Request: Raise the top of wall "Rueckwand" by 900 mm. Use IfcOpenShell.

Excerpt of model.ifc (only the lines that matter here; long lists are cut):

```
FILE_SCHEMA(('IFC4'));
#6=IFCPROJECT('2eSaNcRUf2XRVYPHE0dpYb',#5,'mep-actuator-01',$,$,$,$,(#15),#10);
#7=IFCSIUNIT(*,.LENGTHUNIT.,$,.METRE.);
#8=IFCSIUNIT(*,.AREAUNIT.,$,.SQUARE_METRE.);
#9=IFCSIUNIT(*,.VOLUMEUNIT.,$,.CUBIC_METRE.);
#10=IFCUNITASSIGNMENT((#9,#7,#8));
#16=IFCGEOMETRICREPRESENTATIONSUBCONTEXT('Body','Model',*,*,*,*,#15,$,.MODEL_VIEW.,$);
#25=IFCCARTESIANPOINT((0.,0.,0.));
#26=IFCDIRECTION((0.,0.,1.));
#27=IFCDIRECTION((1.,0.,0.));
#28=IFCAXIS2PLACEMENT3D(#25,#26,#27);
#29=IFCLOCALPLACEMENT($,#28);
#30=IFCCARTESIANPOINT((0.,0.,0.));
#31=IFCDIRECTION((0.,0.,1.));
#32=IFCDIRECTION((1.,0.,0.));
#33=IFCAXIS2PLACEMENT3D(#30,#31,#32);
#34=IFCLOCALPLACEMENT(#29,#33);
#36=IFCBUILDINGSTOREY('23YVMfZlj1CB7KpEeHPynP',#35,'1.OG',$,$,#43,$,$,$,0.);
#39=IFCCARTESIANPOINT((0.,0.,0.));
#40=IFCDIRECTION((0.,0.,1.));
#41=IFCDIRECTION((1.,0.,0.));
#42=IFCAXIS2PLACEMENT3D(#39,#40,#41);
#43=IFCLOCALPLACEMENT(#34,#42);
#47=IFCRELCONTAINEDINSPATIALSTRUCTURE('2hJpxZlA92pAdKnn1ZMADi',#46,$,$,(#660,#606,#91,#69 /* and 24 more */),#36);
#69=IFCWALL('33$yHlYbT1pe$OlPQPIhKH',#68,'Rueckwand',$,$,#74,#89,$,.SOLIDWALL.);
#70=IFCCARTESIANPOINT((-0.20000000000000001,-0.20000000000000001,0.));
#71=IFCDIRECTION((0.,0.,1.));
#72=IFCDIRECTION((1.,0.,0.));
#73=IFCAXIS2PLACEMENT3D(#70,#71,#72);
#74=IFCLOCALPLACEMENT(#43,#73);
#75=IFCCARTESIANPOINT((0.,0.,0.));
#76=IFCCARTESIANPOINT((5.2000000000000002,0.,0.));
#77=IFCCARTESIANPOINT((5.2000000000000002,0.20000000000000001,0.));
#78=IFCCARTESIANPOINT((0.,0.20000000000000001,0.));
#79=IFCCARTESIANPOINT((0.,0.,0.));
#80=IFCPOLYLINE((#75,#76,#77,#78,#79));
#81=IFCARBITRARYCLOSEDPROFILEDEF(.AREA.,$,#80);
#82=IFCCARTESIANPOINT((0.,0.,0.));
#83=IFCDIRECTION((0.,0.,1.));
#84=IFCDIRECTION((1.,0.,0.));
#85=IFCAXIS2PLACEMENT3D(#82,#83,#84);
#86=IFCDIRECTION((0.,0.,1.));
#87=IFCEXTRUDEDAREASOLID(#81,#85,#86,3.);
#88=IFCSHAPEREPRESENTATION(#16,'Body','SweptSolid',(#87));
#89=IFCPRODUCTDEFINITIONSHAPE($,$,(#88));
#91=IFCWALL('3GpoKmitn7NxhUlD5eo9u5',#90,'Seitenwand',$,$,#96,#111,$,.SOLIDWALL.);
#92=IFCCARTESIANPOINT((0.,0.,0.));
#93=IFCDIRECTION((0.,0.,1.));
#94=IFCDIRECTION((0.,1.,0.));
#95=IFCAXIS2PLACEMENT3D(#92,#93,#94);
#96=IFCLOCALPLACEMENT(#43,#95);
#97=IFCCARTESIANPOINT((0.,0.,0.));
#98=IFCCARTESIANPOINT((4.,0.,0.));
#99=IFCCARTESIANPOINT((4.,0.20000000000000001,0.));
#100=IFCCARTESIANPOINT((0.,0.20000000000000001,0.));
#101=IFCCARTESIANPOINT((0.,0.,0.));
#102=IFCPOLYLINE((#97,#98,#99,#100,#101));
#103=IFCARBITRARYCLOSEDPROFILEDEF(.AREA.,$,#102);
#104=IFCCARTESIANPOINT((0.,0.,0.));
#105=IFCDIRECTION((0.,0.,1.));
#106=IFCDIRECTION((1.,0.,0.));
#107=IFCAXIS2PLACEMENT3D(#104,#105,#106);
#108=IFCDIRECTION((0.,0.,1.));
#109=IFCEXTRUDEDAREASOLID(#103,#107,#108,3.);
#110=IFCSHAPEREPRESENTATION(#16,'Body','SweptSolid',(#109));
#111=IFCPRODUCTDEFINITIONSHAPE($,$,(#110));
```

```python
import ifcopenshell
import ifcopenshell.geom
import ifcopenshell.util.representation
import ifcopenshell.util.shape

model = ifcopenshell.open("model.ifc")
settings = ifcopenshell.geom.settings()


def volume(element):
    """Net volume in cubic metres, openings subtracted."""
    shape = ifcopenshell.geom.create_shape(settings, element)
    return ifcopenshell.util.shape.get_volume(shape.geometry)


wall = model.by_guid("33$yHlYbT1pe$OlPQPIhKH")
before = volume(wall)

body = ifcopenshell.util.representation.get_representation(wall, "Model", "Body")
solid = body.Items[0]
old_height = solid.Depth
solid.Depth += 0.9
after = volume(wall)

print(f"height {old_height:g} -> {solid.Depth:g}, volume {before:.3f} -> {after:.3f} m3")

model.write("model-out.ifc")
```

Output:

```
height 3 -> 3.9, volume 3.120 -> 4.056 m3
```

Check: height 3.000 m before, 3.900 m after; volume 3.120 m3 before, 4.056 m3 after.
